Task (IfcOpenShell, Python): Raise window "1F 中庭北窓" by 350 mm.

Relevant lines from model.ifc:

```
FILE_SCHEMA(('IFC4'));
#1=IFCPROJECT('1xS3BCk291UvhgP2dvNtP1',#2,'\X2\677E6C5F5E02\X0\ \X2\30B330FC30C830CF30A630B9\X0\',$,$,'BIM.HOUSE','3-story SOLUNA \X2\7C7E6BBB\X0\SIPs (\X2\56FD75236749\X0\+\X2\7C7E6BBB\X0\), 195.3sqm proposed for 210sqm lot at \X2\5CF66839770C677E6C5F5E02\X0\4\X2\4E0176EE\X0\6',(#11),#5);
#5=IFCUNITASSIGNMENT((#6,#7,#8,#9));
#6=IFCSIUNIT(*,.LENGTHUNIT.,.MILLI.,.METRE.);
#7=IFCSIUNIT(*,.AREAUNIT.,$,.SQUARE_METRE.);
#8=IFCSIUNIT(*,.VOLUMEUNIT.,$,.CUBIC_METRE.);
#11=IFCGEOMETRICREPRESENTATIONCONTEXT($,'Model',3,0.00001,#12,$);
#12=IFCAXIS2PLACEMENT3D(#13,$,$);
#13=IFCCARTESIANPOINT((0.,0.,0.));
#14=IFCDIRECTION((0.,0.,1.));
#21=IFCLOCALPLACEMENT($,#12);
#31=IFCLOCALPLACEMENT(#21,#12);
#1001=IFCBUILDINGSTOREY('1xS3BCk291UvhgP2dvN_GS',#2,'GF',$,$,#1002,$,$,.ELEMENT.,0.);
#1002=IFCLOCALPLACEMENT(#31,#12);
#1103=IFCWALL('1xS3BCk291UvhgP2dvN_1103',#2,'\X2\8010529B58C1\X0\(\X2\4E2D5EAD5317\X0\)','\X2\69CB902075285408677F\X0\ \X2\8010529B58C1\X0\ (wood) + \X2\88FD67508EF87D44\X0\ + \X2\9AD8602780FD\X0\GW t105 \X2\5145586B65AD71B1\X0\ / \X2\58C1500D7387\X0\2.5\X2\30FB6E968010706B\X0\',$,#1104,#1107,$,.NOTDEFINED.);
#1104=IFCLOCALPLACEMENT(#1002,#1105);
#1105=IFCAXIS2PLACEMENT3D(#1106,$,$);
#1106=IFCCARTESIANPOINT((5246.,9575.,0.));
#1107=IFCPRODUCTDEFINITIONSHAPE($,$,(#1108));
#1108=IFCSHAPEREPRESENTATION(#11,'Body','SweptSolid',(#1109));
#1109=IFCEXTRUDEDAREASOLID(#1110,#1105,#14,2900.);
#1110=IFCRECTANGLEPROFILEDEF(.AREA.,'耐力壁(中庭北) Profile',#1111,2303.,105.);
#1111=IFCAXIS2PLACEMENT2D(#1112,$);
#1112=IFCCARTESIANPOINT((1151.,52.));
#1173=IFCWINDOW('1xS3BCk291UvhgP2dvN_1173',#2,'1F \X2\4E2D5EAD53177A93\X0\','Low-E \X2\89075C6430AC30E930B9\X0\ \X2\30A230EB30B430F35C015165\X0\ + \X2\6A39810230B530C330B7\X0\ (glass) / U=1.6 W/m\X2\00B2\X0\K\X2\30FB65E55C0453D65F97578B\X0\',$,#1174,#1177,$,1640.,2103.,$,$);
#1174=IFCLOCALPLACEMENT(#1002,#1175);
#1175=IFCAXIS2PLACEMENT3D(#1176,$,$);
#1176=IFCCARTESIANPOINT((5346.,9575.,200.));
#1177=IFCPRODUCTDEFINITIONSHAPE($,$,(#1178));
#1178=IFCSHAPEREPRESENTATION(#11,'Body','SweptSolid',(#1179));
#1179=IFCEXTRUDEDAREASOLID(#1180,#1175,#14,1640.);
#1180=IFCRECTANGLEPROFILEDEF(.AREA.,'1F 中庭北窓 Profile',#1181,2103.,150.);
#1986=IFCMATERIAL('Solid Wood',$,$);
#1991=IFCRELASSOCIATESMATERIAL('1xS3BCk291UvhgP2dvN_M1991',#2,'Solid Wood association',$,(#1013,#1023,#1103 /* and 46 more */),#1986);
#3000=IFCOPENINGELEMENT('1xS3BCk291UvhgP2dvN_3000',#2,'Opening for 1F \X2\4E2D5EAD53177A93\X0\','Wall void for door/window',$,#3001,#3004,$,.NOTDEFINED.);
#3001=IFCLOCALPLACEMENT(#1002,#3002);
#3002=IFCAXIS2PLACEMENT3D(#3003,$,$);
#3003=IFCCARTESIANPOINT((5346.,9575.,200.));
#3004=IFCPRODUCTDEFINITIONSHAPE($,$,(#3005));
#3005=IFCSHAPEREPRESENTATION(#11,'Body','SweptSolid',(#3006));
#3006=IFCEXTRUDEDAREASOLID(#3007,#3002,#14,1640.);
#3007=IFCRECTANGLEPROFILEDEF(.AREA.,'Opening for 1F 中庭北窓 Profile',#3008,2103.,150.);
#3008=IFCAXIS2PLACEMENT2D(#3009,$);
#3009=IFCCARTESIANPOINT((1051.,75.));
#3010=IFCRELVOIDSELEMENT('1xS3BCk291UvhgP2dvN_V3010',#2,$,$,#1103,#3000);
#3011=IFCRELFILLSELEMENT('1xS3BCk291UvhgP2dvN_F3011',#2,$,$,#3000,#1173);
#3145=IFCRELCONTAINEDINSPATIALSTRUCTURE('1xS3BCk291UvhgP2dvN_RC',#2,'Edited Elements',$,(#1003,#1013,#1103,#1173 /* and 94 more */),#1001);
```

```python
import numpy as np
import ifcopenshell
import ifcopenshell.api.geometry
import ifcopenshell.util.placement
import ifcopenshell.util.unit

model = ifcopenshell.open("model.ifc")
unit_scale = ifcopenshell.util.unit.calculate_unit_scale(model)

window = model.by_id(1173)
opening = window.FillsVoids[0].RelatingOpeningElement
dz = 350.0

shift = np.array([0.0, 0.0, dz])
# The window is not placed relative to its opening, so move both.
for product in (opening, window):
    matrix = ifcopenshell.util.placement.get_local_placement(product.ObjectPlacement)
    matrix[:3, 3] += shift
    ifcopenshell.api.geometry.edit_object_placement(model, product=product, matrix=matrix, is_si=False)

print(f"moved by {dz * unit_scale:+.3f} m")

model.write("model_edited.ifc")
```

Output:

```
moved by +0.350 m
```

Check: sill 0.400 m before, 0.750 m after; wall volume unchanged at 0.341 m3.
